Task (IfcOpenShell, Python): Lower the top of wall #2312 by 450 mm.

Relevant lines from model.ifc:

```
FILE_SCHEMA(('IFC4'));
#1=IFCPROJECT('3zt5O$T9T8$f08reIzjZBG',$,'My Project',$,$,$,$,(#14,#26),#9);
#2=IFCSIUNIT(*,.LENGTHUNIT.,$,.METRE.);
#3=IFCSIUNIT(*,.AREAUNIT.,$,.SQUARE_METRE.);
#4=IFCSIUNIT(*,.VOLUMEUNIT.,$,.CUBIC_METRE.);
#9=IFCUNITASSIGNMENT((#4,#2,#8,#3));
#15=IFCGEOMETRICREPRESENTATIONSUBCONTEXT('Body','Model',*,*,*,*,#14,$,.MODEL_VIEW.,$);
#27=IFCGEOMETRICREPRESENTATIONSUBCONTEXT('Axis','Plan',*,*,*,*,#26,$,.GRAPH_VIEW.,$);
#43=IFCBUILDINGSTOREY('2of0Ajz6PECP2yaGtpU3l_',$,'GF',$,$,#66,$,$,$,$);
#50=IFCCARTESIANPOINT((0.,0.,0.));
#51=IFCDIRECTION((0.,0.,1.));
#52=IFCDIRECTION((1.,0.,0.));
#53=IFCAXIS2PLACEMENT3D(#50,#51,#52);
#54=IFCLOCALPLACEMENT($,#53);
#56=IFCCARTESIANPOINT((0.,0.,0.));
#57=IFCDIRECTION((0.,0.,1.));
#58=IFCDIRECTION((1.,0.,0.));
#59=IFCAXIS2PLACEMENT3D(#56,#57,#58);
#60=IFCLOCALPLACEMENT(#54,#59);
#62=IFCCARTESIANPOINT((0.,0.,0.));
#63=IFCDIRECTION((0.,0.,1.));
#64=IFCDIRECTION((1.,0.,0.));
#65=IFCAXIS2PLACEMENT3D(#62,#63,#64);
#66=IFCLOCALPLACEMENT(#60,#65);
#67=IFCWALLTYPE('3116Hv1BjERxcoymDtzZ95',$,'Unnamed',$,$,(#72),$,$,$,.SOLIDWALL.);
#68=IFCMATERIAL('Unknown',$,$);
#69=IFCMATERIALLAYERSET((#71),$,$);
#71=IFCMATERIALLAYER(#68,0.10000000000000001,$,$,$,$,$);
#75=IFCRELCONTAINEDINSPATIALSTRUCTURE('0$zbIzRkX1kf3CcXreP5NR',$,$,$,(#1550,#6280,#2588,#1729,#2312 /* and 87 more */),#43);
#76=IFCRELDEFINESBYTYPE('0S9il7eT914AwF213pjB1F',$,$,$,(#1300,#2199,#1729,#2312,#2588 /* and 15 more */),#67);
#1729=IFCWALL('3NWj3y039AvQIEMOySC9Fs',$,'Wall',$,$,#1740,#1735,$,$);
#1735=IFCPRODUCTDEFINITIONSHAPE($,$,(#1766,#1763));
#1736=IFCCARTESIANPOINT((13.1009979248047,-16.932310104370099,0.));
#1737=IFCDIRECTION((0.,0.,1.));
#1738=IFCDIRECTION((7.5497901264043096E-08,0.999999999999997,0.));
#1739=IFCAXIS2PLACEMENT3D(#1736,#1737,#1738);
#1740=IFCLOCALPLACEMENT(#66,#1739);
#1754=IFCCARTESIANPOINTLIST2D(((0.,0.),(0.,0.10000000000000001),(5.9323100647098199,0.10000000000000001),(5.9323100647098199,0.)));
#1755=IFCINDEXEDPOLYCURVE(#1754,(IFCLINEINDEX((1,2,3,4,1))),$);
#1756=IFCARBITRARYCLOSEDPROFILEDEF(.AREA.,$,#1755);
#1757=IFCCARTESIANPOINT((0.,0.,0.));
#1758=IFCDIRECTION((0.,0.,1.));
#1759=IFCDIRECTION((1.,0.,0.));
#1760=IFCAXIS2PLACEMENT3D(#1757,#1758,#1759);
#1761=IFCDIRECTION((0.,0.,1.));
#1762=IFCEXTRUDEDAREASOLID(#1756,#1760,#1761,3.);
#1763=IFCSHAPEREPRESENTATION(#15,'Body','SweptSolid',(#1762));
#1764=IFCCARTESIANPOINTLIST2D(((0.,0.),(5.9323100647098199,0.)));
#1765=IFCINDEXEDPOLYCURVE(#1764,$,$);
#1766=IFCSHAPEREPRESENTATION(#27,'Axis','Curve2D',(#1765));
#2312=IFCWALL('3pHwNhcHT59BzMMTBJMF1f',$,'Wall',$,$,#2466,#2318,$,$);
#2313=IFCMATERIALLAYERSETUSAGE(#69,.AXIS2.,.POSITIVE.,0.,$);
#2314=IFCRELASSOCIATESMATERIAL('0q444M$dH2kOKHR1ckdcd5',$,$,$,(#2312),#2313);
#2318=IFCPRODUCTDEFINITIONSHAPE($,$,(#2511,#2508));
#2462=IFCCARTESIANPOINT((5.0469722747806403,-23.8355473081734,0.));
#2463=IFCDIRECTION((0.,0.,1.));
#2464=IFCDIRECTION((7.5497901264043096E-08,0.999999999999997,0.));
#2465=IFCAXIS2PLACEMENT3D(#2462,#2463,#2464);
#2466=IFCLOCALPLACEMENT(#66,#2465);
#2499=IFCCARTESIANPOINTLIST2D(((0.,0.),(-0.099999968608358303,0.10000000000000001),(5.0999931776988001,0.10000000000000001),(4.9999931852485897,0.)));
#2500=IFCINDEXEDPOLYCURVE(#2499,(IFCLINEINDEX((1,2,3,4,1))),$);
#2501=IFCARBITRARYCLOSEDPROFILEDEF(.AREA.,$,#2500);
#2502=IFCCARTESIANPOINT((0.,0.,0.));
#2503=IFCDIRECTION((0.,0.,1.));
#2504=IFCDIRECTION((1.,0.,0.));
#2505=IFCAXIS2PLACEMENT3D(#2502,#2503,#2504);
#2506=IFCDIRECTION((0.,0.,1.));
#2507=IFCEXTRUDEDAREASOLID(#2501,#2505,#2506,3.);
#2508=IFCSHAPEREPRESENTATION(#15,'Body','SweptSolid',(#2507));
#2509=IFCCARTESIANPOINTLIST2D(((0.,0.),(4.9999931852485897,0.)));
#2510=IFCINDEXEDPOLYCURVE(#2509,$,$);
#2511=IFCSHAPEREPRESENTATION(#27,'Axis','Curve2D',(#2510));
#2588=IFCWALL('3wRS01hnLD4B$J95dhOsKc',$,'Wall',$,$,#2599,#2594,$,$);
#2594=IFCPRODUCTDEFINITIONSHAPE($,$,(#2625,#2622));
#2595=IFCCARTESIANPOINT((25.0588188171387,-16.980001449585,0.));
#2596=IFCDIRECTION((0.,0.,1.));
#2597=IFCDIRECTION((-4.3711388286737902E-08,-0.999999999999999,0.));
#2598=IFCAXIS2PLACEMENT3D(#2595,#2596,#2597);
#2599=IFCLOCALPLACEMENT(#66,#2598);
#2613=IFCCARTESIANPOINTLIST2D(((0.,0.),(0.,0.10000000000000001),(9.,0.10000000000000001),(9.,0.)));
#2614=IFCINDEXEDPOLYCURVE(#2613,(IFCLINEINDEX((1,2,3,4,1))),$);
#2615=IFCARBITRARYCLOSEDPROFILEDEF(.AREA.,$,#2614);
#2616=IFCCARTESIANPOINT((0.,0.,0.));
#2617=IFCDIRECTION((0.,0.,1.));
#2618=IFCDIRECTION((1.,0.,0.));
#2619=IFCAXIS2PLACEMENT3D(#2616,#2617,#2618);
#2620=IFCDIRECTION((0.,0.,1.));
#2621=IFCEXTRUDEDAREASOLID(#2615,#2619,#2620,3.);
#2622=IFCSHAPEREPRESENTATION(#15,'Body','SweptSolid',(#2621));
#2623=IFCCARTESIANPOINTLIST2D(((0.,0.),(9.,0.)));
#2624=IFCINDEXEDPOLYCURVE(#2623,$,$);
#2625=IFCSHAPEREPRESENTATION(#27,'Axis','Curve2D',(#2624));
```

```python
import ifcopenshell
import ifcopenshell.geom
import ifcopenshell.util.representation
import ifcopenshell.util.shape

model = ifcopenshell.open("model.ifc")
settings = ifcopenshell.geom.settings()


def volume(element):
    """Net volume in cubic metres, openings subtracted."""
    shape = ifcopenshell.geom.create_shape(settings, element)
    return ifcopenshell.util.shape.get_volume(shape.geometry)


wall = model.by_id(2312)
before = volume(wall)

body = ifcopenshell.util.representation.get_representation(wall, "Model", "Body")
solid = body.Items[0]
old_height = solid.Depth
solid.Depth -= 0.45
after = volume(wall)

print(f"height {old_height:g} -> {solid.Depth:g}, volume {before:.3f} -> {after:.3f} m3")

model.write("model_v2.ifc")
```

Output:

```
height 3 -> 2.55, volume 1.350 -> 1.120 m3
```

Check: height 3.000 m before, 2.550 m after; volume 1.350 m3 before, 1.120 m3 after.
